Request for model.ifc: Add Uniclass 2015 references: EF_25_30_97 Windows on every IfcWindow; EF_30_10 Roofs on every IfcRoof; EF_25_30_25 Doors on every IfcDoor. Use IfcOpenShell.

First a look at what the model holds.

```python
import ifcopenshell

model = ifcopenshell.open("model.ifc")
print(model.schema)
print("classifications:", [c.Name for c in model.by_type("IfcClassification")])
for ifc_class in ("IfcDoor", "IfcRoof", "IfcStair", "IfcWall", "IfcWindow"):
    print(ifc_class, len(model.by_type(ifc_class)))
```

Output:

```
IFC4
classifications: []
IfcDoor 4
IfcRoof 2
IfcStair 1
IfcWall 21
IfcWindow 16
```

```python
import ifcopenshell
import ifcopenshell.api.classification

model = ifcopenshell.open("model.ifc")

system = ifcopenshell.api.classification.add_classification(model, classification="Uniclass 2015")

codes = {
    "IfcWindow": ("EF_25_30_97", "Windows"),
    "IfcRoof": ("EF_30_10", "Roofs"),
    "IfcDoor": ("EF_25_30_25", "Doors"),
}
for ifc_class, (code, name) in codes.items():
    products = model.by_type(ifc_class)
    ifcopenshell.api.classification.add_reference(
        model, products=products, classification=system, identification=code, name=name
    )
    print(code, len(products))

model.write("model-out.ifc")
```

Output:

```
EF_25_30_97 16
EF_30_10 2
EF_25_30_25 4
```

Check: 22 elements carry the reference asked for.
